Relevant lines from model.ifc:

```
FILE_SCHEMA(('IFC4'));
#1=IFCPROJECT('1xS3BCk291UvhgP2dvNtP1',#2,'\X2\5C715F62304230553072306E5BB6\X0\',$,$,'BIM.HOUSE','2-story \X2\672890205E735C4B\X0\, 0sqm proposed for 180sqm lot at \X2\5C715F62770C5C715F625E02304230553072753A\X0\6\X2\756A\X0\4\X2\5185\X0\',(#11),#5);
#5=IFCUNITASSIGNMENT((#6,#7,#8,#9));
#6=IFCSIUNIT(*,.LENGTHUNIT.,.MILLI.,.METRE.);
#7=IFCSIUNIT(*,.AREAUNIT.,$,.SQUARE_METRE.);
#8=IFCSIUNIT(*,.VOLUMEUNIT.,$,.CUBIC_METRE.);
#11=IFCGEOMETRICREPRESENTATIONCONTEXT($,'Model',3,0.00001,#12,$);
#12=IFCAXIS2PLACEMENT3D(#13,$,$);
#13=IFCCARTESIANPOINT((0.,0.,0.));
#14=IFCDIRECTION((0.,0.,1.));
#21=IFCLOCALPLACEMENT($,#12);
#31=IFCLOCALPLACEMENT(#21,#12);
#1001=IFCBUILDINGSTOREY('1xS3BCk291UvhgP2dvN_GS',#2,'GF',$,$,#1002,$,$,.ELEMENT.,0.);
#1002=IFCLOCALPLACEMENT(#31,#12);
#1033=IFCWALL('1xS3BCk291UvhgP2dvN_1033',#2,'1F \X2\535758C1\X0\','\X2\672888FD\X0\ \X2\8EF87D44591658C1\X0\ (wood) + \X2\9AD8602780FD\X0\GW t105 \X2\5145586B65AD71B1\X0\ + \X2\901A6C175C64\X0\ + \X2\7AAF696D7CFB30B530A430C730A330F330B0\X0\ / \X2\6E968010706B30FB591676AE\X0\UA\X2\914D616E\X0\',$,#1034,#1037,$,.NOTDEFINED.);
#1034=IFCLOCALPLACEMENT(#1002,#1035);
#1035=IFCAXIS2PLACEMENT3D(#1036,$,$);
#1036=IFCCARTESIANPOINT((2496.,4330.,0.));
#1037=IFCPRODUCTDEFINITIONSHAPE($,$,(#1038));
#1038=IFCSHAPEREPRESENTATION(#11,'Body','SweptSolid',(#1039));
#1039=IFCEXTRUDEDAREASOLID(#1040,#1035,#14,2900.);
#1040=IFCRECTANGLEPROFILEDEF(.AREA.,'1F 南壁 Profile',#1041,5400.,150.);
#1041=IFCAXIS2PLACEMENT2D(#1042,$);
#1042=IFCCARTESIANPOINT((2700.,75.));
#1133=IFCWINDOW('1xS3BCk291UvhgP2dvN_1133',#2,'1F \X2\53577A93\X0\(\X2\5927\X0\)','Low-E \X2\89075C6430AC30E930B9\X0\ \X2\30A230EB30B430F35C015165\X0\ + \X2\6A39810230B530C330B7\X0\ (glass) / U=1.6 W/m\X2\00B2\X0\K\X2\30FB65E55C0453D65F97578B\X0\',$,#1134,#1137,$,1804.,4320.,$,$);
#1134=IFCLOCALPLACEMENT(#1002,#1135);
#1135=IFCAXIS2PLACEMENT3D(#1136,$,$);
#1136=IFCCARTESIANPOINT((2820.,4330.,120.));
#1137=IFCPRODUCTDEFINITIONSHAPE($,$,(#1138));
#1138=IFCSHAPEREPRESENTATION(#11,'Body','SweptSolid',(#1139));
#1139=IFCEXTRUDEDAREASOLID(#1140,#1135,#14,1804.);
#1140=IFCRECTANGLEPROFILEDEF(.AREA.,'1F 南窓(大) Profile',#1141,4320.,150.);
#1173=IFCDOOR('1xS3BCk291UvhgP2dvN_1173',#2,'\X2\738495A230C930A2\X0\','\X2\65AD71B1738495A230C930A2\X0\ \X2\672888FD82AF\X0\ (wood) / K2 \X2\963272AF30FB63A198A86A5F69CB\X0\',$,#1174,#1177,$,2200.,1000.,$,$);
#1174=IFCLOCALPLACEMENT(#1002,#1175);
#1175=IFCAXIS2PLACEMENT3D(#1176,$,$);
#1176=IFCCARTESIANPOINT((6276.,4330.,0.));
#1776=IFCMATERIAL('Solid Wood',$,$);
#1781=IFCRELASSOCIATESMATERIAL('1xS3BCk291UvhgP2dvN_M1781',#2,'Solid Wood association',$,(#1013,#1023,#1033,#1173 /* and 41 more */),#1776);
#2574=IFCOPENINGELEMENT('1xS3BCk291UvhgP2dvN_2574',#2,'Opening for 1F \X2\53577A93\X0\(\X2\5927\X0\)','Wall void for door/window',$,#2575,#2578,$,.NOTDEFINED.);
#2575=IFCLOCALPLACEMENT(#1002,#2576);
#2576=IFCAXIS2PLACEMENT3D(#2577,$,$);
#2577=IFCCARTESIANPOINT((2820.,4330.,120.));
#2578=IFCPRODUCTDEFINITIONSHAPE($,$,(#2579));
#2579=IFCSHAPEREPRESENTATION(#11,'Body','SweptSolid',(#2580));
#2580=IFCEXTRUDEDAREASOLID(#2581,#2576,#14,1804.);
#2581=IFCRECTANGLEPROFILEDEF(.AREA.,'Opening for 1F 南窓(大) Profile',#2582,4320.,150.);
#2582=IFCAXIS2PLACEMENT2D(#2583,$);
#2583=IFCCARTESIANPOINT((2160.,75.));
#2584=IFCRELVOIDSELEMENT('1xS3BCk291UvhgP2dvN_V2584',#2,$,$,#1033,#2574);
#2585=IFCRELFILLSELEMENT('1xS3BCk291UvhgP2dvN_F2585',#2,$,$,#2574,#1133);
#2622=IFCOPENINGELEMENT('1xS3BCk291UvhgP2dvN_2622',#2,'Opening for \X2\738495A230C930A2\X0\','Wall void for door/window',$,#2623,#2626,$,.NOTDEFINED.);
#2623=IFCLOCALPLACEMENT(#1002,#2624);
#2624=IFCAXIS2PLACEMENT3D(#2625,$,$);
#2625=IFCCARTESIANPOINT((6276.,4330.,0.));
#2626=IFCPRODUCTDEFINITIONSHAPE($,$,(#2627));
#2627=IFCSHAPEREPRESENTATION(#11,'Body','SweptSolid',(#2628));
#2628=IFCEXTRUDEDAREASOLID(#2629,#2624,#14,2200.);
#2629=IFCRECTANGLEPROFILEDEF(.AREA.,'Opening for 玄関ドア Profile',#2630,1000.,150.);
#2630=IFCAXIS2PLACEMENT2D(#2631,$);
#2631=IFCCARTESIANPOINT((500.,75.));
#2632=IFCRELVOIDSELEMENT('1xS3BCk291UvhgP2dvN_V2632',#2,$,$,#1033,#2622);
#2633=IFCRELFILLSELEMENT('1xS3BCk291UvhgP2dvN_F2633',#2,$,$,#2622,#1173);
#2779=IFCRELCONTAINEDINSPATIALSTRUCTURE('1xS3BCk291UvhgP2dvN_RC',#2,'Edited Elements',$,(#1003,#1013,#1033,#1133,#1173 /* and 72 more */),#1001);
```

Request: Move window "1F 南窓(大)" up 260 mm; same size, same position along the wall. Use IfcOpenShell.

```python
import numpy as np
import ifcopenshell
import ifcopenshell.api.geometry
import ifcopenshell.util.placement
import ifcopenshell.util.unit

model = ifcopenshell.open("model.ifc")
unit_scale = ifcopenshell.util.unit.calculate_unit_scale(model)

window = model.by_guid("1xS3BCk291UvhgP2dvN_1133")
opening = window.FillsVoids[0].RelatingOpeningElement
dz = 260.0

shift = np.array([0.0, 0.0, dz])
# The window is not placed relative to its opening, so move both.
for product in (opening, window):
    matrix = ifcopenshell.util.placement.get_local_placement(product.ObjectPlacement)
    matrix[:3, 3] += shift
    ifcopenshell.api.geometry.edit_object_placement(model, product=product, matrix=matrix, is_si=False)

print(f"moved by {dz * unit_scale:+.3f} m")

model.write("model-out.ifc")
```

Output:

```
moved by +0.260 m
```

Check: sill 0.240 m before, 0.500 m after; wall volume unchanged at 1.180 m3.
